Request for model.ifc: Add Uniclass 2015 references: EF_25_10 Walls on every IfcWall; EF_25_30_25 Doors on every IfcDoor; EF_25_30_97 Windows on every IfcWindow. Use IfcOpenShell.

First a look at what the model holds.

```python
import ifcopenshell

model = ifcopenshell.open("model.ifc")
print(model.schema)
print("classifications:", [c.Name for c in model.by_type("IfcClassification")])
for ifc_class in ("IfcDoor", "IfcRoof", "IfcStair", "IfcWall", "IfcWindow"):
    print(ifc_class, len(model.by_type(ifc_class)))
```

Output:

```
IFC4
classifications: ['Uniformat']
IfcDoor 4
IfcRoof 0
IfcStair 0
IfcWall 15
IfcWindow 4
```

```python
import ifcopenshell
import ifcopenshell.api.classification

model = ifcopenshell.open("model.ifc")

system = ifcopenshell.api.classification.add_classification(model, classification="Uniclass 2015")

codes = {
    "IfcWall": ("EF_25_10", "Walls"),
    "IfcDoor": ("EF_25_30_25", "Doors"),
    "IfcWindow": ("EF_25_30_97", "Windows"),
}
for ifc_class, (code, name) in codes.items():
    products = model.by_type(ifc_class)
    ifcopenshell.api.classification.add_reference(
        model, products=products, classification=system, identification=code, name=name
    )
    print(code, len(products))

model.write("model_edited.ifc")
```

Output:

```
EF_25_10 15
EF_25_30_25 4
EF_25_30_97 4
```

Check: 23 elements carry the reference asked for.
